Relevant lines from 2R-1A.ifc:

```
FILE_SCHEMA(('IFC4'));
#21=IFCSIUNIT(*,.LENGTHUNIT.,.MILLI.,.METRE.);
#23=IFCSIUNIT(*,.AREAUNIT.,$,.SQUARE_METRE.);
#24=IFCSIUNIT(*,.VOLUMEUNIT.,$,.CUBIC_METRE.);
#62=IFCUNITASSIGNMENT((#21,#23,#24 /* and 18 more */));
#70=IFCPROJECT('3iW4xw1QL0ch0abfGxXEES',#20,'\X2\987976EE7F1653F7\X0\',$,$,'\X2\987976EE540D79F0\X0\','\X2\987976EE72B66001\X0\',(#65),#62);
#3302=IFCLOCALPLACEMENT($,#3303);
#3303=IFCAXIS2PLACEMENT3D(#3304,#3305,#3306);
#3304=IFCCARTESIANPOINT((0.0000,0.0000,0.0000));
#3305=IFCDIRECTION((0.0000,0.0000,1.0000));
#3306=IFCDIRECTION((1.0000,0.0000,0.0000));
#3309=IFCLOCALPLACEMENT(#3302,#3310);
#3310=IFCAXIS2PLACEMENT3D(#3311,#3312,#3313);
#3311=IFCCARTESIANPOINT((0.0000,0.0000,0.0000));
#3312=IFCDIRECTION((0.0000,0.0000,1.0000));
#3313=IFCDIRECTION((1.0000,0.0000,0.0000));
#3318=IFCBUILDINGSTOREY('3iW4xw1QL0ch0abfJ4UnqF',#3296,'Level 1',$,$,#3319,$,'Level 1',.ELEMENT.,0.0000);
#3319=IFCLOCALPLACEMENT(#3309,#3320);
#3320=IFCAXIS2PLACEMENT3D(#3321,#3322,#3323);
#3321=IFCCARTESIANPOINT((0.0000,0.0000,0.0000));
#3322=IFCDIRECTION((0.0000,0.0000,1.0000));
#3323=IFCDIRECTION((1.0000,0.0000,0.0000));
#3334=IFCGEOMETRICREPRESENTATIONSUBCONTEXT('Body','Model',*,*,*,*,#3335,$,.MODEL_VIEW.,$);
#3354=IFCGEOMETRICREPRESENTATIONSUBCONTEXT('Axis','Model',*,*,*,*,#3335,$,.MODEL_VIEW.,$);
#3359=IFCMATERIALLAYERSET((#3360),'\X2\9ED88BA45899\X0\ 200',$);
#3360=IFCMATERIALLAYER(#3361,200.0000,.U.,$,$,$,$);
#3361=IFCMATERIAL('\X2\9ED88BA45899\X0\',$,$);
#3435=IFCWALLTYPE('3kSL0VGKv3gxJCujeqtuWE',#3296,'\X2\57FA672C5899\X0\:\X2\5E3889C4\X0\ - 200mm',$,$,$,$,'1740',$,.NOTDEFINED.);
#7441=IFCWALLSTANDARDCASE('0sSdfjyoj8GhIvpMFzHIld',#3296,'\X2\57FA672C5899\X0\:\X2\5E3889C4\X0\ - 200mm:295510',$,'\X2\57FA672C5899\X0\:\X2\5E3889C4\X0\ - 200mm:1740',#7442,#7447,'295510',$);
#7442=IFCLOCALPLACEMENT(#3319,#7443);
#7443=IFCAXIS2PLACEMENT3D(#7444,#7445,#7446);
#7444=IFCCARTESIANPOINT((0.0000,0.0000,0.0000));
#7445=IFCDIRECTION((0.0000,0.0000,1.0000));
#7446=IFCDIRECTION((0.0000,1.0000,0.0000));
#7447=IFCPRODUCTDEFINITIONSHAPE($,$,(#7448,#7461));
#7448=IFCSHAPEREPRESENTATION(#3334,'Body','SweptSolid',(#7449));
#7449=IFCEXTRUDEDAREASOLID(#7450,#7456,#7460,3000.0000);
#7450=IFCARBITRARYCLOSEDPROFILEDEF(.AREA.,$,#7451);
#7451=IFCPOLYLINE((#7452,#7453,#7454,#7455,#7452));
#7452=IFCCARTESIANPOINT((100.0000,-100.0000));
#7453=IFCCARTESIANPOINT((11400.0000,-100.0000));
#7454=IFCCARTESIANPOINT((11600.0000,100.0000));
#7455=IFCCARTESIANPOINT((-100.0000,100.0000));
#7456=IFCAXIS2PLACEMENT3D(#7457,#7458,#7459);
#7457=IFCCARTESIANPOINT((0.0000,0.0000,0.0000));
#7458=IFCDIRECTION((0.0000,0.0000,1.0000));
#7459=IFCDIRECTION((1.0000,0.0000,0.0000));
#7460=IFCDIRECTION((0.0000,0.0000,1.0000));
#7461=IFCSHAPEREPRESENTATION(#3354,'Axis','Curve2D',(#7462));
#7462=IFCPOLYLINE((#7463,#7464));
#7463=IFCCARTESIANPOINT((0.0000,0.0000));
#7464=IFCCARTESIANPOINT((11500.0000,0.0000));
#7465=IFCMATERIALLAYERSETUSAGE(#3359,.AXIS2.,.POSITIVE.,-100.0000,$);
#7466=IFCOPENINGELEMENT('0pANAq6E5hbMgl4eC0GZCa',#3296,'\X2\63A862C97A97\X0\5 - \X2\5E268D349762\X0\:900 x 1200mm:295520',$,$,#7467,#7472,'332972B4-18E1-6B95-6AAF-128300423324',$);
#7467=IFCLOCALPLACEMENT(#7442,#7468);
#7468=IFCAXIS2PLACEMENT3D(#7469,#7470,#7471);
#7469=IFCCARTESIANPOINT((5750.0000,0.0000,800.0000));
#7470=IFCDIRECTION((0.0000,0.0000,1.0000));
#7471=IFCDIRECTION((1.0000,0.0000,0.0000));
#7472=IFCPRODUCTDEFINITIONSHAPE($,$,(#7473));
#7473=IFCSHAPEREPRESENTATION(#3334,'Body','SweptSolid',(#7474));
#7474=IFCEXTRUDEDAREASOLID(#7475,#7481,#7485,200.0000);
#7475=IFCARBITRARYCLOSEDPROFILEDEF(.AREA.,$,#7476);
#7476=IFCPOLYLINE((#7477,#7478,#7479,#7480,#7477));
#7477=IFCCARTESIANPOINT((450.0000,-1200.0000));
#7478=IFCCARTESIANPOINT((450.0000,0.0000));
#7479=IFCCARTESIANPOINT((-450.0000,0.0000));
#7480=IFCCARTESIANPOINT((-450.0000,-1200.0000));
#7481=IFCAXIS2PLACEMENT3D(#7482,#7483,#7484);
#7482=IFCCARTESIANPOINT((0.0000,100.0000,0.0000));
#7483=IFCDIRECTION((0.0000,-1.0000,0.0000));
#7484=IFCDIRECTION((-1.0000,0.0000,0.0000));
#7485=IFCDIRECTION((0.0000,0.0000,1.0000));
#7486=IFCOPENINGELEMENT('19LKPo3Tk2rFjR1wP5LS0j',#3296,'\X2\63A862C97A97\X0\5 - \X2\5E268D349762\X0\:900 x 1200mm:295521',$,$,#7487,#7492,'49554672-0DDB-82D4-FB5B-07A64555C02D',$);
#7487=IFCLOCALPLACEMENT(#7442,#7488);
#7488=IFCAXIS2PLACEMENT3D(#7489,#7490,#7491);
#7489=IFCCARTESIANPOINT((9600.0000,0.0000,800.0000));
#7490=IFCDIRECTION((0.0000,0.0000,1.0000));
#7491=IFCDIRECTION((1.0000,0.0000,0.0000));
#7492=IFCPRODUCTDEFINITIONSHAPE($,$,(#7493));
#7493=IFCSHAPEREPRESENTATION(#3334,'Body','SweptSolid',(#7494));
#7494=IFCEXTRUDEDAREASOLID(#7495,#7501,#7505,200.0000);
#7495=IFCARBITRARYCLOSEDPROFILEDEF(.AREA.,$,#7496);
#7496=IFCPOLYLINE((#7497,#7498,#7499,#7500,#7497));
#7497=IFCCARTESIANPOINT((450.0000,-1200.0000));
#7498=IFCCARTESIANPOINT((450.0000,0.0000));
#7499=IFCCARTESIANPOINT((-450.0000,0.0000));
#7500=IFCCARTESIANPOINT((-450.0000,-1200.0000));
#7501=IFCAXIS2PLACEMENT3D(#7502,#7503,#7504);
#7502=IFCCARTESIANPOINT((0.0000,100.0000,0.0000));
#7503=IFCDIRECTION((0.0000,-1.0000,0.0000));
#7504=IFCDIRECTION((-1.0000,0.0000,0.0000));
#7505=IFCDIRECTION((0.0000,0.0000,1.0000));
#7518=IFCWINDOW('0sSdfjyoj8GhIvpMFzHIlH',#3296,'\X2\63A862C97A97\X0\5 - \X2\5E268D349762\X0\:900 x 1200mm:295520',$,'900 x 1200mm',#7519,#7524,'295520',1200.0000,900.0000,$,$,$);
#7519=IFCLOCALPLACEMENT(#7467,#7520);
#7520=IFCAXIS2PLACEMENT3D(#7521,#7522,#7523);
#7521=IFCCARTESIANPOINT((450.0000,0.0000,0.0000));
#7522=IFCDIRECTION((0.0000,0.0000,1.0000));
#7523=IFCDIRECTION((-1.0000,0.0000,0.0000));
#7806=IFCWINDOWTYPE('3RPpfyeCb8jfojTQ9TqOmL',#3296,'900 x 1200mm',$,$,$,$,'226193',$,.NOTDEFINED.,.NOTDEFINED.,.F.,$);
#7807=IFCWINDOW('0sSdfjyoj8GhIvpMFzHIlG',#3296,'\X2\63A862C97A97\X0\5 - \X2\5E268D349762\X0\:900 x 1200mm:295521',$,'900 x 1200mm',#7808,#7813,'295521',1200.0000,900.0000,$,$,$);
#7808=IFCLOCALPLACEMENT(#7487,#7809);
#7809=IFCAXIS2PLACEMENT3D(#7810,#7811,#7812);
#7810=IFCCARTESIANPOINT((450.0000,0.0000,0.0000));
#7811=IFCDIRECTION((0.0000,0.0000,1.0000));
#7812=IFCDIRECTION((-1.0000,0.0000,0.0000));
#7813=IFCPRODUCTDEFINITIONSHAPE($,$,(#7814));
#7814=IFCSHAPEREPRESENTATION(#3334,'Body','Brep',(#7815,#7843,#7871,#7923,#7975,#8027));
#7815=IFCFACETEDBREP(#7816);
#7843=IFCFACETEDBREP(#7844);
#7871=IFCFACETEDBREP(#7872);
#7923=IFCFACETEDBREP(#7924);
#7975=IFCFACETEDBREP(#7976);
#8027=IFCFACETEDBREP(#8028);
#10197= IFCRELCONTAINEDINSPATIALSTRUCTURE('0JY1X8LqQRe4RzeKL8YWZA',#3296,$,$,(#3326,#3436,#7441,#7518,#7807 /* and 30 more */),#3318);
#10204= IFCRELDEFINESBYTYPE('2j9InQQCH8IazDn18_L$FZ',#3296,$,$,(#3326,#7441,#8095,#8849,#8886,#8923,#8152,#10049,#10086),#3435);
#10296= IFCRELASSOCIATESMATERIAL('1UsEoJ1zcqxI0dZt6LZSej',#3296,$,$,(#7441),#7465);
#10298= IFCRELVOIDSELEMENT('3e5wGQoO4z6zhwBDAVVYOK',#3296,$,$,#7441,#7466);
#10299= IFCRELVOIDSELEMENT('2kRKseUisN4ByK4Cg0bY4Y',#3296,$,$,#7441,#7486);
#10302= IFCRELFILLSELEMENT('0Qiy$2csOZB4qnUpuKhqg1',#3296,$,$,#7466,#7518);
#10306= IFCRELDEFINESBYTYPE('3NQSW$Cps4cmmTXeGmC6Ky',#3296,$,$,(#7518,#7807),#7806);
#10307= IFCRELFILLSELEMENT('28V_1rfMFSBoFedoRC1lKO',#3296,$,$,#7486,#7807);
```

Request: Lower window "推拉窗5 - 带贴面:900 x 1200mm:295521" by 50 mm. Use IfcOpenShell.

```python
import numpy as np
import ifcopenshell
import ifcopenshell.api.geometry
import ifcopenshell.util.placement
import ifcopenshell.util.unit

model = ifcopenshell.open("2R-1A.ifc")
unit_scale = ifcopenshell.util.unit.calculate_unit_scale(model)

window = model.by_guid("0sSdfjyoj8GhIvpMFzHIlG")
opening = window.FillsVoids[0].RelatingOpeningElement
dz = -50.0

shift = np.array([0.0, 0.0, dz])
# The window is placed relative to its opening, so it follows when the opening moves.
matrix = ifcopenshell.util.placement.get_local_placement(opening.ObjectPlacement)
matrix[:3, 3] += shift
ifcopenshell.api.geometry.edit_object_placement(
    model, product=opening, matrix=matrix, is_si=False, should_transform_children=True
)

print(f"moved by {dz * unit_scale:+.3f} m")

model.write("2R-1A-out.ifc")
```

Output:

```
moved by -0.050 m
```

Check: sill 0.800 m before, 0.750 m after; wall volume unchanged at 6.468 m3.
